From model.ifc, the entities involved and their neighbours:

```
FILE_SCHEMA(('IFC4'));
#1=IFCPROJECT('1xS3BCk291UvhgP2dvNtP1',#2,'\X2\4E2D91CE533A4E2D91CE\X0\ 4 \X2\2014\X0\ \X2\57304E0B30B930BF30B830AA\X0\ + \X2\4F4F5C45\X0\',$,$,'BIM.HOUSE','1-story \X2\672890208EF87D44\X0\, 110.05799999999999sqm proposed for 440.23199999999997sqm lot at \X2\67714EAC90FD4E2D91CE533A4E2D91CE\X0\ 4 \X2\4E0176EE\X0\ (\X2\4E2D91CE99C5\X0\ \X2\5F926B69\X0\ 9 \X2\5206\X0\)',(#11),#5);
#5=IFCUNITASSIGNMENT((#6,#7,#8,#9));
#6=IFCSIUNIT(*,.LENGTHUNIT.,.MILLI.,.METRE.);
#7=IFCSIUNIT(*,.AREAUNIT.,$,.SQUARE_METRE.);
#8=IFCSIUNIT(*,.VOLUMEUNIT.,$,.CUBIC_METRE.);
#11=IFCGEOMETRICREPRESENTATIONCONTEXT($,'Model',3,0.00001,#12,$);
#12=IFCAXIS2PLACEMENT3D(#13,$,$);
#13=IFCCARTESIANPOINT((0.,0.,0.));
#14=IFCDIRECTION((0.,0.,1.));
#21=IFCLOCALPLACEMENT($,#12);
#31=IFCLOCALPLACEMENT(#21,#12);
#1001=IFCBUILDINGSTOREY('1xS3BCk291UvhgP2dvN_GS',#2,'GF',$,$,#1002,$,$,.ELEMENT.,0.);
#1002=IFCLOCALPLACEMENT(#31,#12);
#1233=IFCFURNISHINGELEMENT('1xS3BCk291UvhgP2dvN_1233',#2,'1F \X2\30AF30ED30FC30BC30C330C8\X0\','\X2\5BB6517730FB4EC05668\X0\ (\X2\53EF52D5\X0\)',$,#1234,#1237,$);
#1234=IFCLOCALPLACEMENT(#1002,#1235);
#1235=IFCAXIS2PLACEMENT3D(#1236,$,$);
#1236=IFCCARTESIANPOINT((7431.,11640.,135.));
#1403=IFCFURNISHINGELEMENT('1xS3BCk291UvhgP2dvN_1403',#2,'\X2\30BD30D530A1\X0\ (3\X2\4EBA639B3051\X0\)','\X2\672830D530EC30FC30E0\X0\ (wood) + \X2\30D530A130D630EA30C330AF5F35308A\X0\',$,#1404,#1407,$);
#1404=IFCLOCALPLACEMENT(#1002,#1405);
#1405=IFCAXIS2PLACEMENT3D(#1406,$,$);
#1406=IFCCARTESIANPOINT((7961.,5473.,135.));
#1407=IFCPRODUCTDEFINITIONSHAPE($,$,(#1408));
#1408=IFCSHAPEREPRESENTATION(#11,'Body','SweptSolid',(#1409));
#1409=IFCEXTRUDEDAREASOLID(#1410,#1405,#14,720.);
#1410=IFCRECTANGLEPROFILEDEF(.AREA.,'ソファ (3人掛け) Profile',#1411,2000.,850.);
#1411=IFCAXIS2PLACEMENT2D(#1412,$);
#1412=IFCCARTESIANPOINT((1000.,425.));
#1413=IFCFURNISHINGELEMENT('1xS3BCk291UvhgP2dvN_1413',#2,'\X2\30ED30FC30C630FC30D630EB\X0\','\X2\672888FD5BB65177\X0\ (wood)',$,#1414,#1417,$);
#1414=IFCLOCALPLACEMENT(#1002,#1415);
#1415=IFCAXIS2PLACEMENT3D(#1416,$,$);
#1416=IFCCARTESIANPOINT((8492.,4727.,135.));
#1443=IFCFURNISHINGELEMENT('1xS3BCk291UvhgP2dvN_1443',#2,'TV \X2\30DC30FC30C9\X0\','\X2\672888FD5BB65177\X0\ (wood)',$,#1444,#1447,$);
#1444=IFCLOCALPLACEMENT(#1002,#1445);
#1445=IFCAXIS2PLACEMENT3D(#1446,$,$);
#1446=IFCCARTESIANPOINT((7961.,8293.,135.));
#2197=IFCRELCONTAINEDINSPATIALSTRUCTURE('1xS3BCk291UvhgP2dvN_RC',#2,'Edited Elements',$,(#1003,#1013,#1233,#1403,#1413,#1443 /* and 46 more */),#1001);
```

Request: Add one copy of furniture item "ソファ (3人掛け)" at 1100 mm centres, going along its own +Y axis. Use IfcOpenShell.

```python
import ifcopenshell
import ifcopenshell.api.geometry
import ifcopenshell.api.root
import ifcopenshell.util.element
import ifcopenshell.util.placement
import ifcopenshell.util.unit

model = ifcopenshell.open("model.ifc")
unit_scale = ifcopenshell.util.unit.calculate_unit_scale(model)


def reuse_history(source, copy):
    """copy_class also copies each property set's owner history, people and application; keep the originals."""
    for rel in copy.IsDefinedBy:
        if rel.is_a("IfcRelDefinesByProperties") and (history := rel.RelatingPropertyDefinition.OwnerHistory):
            rel.RelatingPropertyDefinition.OwnerHistory = source.OwnerHistory
            ifcopenshell.util.element.remove_deep2(model, history)


source = model.by_id(1403)
base = ifcopenshell.util.placement.get_local_placement(source.ObjectPlacement)
step = base[:3, 1] * 1.1 / unit_scale

for i in range(1, 2):
    copy = ifcopenshell.api.root.copy_class(model, product=source)
    copy.Representation = ifcopenshell.util.element.copy_deep(
        model, source.Representation, exclude=["IfcGeometricRepresentationContext", "IfcRepresentationMap"]
    )
    reuse_history(source, copy)
    matrix = base.copy()
    matrix[:3, 3] += i * step
    print("added at", matrix[:3, 3].round(3) + 0.0)
    ifcopenshell.api.geometry.edit_object_placement(model, product=copy, matrix=matrix, is_si=False)

model.write("model-out.ifc")
```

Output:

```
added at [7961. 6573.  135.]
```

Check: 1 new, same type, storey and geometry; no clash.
